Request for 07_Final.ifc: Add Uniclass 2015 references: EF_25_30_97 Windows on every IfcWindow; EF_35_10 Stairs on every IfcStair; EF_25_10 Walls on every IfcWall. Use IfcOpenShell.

First a look at what the model holds.

```python
import ifcopenshell

model = ifcopenshell.open("07_Final.ifc")
print(model.schema)
print("classifications:", [c.Name for c in model.by_type("IfcClassification")])
for ifc_class in ("IfcDoor", "IfcRoof", "IfcStair", "IfcWall", "IfcWindow"):
    print(ifc_class, len(model.by_type(ifc_class)))
```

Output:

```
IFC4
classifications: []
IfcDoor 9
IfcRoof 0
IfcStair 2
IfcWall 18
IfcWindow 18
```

```python
import ifcopenshell
import ifcopenshell.api.classification

model = ifcopenshell.open("07_Final.ifc")

system = ifcopenshell.api.classification.add_classification(model, classification="Uniclass 2015")

codes = {
    "IfcWindow": ("EF_25_30_97", "Windows"),
    "IfcStair": ("EF_35_10", "Stairs"),
    "IfcWall": ("EF_25_10", "Walls"),
}
for ifc_class, (code, name) in codes.items():
    products = model.by_type(ifc_class)
    ifcopenshell.api.classification.add_reference(
        model, products=products, classification=system, identification=code, name=name
    )
    print(code, len(products))

model.write("07_Final_edited.ifc")
```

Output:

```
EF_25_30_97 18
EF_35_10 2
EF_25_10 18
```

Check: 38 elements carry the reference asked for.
